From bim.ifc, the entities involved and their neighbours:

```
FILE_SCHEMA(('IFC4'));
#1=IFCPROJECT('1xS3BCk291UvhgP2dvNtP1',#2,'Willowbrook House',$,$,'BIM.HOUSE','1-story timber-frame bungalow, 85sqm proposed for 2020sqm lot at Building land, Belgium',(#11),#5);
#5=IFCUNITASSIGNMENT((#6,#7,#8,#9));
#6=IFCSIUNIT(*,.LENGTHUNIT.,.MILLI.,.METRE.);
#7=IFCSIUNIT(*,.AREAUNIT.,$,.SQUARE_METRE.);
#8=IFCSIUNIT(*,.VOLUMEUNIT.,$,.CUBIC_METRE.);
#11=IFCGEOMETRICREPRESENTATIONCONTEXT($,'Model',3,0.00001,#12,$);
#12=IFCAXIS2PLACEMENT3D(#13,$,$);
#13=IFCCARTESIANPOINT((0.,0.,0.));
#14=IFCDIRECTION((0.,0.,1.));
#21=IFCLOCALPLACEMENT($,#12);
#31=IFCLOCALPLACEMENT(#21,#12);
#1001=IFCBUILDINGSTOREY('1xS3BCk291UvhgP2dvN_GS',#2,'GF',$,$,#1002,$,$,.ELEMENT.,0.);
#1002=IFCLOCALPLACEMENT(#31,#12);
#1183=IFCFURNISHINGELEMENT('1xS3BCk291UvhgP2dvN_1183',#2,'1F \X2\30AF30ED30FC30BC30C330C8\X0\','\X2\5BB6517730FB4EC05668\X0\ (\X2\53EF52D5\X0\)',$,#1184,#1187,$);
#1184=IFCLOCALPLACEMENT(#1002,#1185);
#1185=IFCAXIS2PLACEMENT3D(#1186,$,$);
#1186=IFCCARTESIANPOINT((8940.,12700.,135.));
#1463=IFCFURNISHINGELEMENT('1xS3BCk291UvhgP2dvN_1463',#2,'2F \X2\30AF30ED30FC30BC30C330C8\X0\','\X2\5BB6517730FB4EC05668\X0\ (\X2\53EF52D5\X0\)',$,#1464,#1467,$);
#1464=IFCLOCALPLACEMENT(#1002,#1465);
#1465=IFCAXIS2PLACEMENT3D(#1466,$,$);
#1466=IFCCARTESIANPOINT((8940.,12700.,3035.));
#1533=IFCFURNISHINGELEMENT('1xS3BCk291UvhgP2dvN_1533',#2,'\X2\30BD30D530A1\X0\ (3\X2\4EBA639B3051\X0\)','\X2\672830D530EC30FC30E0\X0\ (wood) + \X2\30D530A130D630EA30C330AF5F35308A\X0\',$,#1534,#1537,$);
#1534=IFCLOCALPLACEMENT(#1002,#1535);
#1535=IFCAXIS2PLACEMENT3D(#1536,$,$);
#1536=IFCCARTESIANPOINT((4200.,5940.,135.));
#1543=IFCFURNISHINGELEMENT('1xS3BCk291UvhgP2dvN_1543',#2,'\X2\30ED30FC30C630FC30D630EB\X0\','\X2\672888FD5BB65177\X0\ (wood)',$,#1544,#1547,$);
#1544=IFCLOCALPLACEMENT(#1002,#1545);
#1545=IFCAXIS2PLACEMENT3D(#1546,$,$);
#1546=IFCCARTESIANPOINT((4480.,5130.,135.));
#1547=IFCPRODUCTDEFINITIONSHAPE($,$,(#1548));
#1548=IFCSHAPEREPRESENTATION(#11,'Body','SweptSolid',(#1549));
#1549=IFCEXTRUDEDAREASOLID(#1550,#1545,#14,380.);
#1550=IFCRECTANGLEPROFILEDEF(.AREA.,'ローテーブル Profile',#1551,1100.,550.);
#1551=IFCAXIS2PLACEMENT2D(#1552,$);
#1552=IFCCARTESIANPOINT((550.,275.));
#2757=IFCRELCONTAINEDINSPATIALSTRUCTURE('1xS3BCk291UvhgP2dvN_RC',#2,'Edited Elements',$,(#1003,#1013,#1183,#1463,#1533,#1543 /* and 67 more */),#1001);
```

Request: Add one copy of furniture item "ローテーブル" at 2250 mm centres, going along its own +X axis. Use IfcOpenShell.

```python
import ifcopenshell
import ifcopenshell.api.geometry
import ifcopenshell.api.root
import ifcopenshell.util.element
import ifcopenshell.util.placement
import ifcopenshell.util.unit

model = ifcopenshell.open("bim.ifc")
unit_scale = ifcopenshell.util.unit.calculate_unit_scale(model)


def reuse_history(source, copy):
    """copy_class also copies each property set's owner history, people and application; keep the originals."""
    for rel in copy.IsDefinedBy:
        if rel.is_a("IfcRelDefinesByProperties") and (history := rel.RelatingPropertyDefinition.OwnerHistory):
            rel.RelatingPropertyDefinition.OwnerHistory = source.OwnerHistory
            ifcopenshell.util.element.remove_deep2(model, history)


source = model.by_guid("1xS3BCk291UvhgP2dvN_1543")
base = ifcopenshell.util.placement.get_local_placement(source.ObjectPlacement)
step = base[:3, 0] * 2.25 / unit_scale

for i in range(1, 2):
    copy = ifcopenshell.api.root.copy_class(model, product=source)
    copy.Representation = ifcopenshell.util.element.copy_deep(
        model, source.Representation, exclude=["IfcGeometricRepresentationContext", "IfcRepresentationMap"]
    )
    reuse_history(source, copy)
    matrix = base.copy()
    matrix[:3, 3] += i * step
    print("added at", matrix[:3, 3].round(3) + 0.0)
    ifcopenshell.api.geometry.edit_object_placement(model, product=copy, matrix=matrix, is_si=False)

model.write("bim_edited.ifc")
```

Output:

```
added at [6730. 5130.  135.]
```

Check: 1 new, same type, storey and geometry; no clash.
